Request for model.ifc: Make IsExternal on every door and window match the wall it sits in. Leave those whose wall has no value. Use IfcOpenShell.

First a look at what the model holds.

```python
import ifcopenshell
import ifcopenshell.util.element

model = ifcopenshell.open("model.ifc")
print(model.schema)
seen = {}
for e in model.by_type("IfcDoor") + model.by_type("IfcWindow"):
    if not e.FillsVoids:
        continue
    host = e.FillsVoids[0].RelatingOpeningElement.VoidsElements[0].RelatingBuildingElement
    own = ifcopenshell.util.element.get_pset(e, f"Pset_{e.is_a()[3:].removesuffix('StandardCase')}Common", "IsExternal")
    wall = ifcopenshell.util.element.get_pset(host, "Pset_WallCommon", "IsExternal")
    seen[e.is_a(), own, wall] = seen.get((e.is_a(), own, wall), 0) + 1
for (cls, own, wall), count in sorted(seen.items(), key=str):
    print(count, cls, "IsExternal:", own, "| host wall:", wall)
```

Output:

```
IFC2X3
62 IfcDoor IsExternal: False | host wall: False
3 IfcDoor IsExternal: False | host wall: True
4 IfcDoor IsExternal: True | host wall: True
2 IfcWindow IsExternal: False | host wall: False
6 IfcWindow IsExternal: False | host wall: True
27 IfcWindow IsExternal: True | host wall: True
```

```python
import ifcopenshell
import ifcopenshell.api.pset
import ifcopenshell.util.element

model = ifcopenshell.open("model.ifc")

count = 0
for ifc_class, pset_name in (("IfcDoor", "Pset_DoorCommon"), ("IfcWindow", "Pset_WindowCommon")):
    for e in model.by_type(ifc_class):
        if not e.FillsVoids:
            continue
        host = e.FillsVoids[0].RelatingOpeningElement.VoidsElements[0].RelatingBuildingElement
        external = ifcopenshell.util.element.get_pset(host, "Pset_WallCommon", "IsExternal")
        if external is None or ifcopenshell.util.element.get_pset(e, pset_name, "IsExternal") == external:
            continue
        pset = ifcopenshell.api.pset.add_pset(model, product=e, name=pset_name)
        ifcopenshell.api.pset.edit_pset(model, pset=pset, properties={"IsExternal": external})
        count += 1

print(count, "updated")

model.write("model_rev.ifc")
```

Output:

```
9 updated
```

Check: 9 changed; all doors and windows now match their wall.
